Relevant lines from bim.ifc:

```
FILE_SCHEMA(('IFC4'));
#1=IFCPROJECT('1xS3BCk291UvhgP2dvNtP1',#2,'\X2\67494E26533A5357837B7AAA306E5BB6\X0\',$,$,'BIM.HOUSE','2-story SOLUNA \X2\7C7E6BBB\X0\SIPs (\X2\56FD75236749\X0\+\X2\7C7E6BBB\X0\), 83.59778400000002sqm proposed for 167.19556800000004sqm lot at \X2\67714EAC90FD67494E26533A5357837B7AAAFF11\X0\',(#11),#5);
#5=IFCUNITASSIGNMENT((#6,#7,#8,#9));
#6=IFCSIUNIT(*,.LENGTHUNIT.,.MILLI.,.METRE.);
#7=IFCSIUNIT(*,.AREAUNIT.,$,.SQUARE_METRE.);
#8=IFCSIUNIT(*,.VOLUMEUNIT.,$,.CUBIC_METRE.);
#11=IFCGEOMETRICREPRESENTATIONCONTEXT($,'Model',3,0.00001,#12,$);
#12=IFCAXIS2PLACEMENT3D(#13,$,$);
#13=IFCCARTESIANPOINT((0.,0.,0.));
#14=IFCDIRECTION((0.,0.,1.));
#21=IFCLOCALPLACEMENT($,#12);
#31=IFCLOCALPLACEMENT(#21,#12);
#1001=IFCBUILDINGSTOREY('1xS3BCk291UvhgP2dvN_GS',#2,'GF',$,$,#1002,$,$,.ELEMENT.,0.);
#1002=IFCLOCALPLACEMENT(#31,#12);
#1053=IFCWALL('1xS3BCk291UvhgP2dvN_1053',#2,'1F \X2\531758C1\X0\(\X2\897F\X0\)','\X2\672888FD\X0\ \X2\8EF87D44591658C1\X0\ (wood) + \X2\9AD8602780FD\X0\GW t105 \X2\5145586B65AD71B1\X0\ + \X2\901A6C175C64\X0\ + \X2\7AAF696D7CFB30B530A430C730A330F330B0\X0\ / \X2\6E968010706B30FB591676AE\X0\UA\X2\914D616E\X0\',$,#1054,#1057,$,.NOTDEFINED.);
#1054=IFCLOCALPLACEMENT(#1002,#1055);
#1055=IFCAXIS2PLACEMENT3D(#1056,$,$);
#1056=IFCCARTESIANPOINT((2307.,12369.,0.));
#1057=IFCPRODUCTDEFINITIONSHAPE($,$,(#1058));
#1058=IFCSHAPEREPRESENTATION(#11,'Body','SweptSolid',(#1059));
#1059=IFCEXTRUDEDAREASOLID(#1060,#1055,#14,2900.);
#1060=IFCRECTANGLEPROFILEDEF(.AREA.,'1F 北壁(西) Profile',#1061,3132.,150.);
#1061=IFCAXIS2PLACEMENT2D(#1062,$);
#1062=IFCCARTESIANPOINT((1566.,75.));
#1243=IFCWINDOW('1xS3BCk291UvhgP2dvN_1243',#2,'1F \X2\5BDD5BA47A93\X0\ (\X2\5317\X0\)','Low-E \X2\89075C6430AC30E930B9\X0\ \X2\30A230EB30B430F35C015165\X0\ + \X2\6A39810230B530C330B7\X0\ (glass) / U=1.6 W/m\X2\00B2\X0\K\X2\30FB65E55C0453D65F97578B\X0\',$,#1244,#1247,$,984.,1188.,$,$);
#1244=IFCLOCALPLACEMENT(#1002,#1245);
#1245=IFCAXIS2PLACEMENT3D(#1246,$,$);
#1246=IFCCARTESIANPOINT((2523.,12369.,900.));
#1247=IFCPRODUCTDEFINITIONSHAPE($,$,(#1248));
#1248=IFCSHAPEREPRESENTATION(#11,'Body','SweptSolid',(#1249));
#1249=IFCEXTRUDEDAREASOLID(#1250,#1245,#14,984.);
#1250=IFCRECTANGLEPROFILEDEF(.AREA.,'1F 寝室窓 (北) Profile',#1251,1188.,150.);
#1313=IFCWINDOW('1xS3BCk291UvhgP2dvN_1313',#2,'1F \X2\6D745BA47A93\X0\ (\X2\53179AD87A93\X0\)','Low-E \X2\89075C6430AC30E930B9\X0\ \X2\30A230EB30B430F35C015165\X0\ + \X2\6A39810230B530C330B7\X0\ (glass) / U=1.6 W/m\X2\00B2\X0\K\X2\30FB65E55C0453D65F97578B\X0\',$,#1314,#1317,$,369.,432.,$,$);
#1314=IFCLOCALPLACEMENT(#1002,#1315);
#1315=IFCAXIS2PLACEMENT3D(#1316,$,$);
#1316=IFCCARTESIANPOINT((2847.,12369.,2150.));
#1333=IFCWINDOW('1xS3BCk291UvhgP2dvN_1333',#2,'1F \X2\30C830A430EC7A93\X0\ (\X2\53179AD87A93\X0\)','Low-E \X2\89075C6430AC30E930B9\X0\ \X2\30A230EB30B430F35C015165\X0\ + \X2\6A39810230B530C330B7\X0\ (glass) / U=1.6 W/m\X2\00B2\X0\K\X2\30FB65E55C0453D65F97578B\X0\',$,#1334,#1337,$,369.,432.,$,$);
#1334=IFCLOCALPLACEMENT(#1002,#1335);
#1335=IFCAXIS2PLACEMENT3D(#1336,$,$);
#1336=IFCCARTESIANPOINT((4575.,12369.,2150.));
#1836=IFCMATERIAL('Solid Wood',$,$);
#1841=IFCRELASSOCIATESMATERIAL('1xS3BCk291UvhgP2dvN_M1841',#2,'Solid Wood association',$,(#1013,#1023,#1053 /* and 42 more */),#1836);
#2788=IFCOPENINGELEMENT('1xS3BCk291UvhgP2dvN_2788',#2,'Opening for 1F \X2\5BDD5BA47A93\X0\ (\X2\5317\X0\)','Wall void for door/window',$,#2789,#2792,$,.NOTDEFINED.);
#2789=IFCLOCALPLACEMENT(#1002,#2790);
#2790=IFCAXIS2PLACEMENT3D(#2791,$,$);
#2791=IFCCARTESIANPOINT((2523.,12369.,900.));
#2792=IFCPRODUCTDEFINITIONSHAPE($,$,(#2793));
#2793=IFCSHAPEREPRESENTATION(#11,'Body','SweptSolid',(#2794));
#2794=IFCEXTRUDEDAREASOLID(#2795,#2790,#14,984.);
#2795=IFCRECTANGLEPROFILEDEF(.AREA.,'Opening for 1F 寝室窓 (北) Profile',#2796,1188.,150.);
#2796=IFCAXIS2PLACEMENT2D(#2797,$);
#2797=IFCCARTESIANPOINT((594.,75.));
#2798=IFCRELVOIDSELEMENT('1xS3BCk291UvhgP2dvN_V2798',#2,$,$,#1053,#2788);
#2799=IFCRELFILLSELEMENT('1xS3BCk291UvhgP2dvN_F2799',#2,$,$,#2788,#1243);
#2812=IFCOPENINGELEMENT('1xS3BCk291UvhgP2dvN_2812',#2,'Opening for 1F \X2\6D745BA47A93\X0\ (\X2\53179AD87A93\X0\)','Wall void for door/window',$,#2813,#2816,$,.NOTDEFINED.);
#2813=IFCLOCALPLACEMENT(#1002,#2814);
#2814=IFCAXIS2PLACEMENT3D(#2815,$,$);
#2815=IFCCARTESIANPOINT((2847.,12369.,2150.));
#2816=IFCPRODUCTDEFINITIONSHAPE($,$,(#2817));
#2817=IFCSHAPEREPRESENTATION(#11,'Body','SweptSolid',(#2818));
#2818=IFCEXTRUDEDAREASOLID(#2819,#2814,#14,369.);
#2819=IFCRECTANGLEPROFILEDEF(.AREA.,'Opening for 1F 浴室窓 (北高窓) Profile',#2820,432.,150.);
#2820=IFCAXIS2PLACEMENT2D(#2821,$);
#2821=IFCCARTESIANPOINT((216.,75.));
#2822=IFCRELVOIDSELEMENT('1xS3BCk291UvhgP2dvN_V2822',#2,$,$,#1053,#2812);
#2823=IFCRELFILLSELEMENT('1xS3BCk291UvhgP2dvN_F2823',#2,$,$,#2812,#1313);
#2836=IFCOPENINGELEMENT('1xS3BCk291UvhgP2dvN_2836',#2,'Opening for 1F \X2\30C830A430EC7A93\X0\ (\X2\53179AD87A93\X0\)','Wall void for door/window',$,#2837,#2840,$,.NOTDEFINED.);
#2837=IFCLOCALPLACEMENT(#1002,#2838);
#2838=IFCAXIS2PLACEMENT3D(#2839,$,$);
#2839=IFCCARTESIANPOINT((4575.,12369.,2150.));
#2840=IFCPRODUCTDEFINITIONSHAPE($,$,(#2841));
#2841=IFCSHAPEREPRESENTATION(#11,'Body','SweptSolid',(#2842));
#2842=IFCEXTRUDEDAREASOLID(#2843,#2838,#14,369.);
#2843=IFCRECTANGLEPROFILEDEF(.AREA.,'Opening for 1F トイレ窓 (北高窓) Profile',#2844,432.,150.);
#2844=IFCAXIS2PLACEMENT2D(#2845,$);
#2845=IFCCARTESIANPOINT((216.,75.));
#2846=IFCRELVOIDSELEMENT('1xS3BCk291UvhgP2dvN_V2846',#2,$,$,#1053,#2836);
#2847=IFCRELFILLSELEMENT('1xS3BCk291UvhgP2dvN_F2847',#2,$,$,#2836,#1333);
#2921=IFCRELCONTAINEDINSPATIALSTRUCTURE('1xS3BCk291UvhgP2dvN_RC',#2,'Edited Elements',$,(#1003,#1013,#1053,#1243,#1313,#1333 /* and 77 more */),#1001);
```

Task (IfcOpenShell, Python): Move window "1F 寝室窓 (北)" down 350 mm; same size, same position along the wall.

```python
import numpy as np
import ifcopenshell
import ifcopenshell.api.geometry
import ifcopenshell.util.placement
import ifcopenshell.util.unit

model = ifcopenshell.open("bim.ifc")
unit_scale = ifcopenshell.util.unit.calculate_unit_scale(model)

window = model.by_guid("1xS3BCk291UvhgP2dvN_1243")
opening = window.FillsVoids[0].RelatingOpeningElement
dz = -0.35 / unit_scale

shift = np.array([0.0, 0.0, dz])
# The window is not placed relative to its opening, so move both.
for product in (opening, window):
    matrix = ifcopenshell.util.placement.get_local_placement(product.ObjectPlacement)
    matrix[:3, 3] += shift
    ifcopenshell.api.geometry.edit_object_placement(model, product=product, matrix=matrix, is_si=False)

print(f"moved by {dz * unit_scale:+.3f} m")

model.write("bim-out.ifc")
```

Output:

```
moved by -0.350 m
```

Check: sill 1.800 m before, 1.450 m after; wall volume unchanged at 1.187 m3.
